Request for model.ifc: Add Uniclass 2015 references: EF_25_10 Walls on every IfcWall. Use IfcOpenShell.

First a look at what the model holds.

```python
import ifcopenshell

model = ifcopenshell.open("model.ifc")
print(model.schema)
print("classifications:", [c.Name for c in model.by_type("IfcClassification")])
for ifc_class in ("IfcDoor", "IfcRoof", "IfcStair", "IfcWall", "IfcWindow"):
    print(ifc_class, len(model.by_type(ifc_class)))
```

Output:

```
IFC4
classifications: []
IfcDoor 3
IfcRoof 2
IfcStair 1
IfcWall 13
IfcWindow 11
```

```python
import ifcopenshell
import ifcopenshell.api.classification

model = ifcopenshell.open("model.ifc")

system = ifcopenshell.api.classification.add_classification(model, classification="Uniclass 2015")

codes = {
    "IfcWall": ("EF_25_10", "Walls"),
}
for ifc_class, (code, name) in codes.items():
    products = model.by_type(ifc_class)
    ifcopenshell.api.classification.add_reference(
        model, products=products, classification=system, identification=code, name=name
    )
    print(code, len(products))

model.write("model_v2.ifc")
```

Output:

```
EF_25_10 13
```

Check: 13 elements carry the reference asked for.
